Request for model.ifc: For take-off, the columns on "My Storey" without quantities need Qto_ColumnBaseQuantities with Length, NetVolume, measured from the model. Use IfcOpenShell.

First a look at what the model holds.

```python
import ifcopenshell
import ifcopenshell.util.element
import ifcopenshell.util.unit

model = ifcopenshell.open("model.ifc")
print(model.schema)
for unit_type in ("LENGTHUNIT", "AREAUNIT", "VOLUMEUNIT"):
    print(unit_type, ifcopenshell.util.unit.calculate_unit_scale(model, unit_type))
storey = next(s for s in model.by_type("IfcBuildingStorey") if s.Name == "My Storey")
columns = [e for e in ifcopenshell.util.element.get_decomposition(storey) if e.is_a("IfcColumn")]
for e in sorted(columns, key=lambda e: e.id()):
    print(e.id(), e.is_a(), e.Name, list(ifcopenshell.util.element.get_psets(e, qtos_only=True)), sep=" | ")
```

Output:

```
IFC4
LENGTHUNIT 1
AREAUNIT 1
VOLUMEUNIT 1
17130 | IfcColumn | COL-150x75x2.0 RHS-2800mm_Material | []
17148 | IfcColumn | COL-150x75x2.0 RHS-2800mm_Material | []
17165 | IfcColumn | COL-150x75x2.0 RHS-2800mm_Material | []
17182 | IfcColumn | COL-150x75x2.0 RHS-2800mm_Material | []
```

```python
import ifcopenshell
import ifcopenshell.api.pset
import ifcopenshell.geom
import ifcopenshell.util.element
import ifcopenshell.util.shape
import ifcopenshell.util.unit

model = ifcopenshell.open("model.ifc")
unit_scale = ifcopenshell.util.unit.calculate_unit_scale(model)
volume_scale = ifcopenshell.util.unit.calculate_unit_scale(model, "VOLUMEUNIT")
settings = ifcopenshell.geom.settings()

storey = next(s for s in model.by_type("IfcBuildingStorey") if s.Name == "My Storey")
columns = [e for e in ifcopenshell.util.element.get_decomposition(storey) if e.is_a("IfcColumn")]

for e in sorted(columns, key=lambda e: e.id()):
    if ifcopenshell.util.element.get_psets(e, qtos_only=True, should_inherit=False):
        continue
    # Geometry comes back in metres, in the element's own axes.
    shape = ifcopenshell.geom.create_shape(settings, e)
    values = {
        "Length": ifcopenshell.util.shape.get_z(shape.geometry) / unit_scale,
        "NetVolume": ifcopenshell.util.shape.get_volume(shape.geometry) / volume_scale,
    }
    qto = ifcopenshell.api.pset.add_qto(model, product=e, name="Qto_ColumnBaseQuantities")
    ifcopenshell.api.pset.edit_qto(model, qto=qto, properties=values)
    print(e.id(), {k: round(v, 3) for k, v in values.items()})

model.write("model-out.ifc")
```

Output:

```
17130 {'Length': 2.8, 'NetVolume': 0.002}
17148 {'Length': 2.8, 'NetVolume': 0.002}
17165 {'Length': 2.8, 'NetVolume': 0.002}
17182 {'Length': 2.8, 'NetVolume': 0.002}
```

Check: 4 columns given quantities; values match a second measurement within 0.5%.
